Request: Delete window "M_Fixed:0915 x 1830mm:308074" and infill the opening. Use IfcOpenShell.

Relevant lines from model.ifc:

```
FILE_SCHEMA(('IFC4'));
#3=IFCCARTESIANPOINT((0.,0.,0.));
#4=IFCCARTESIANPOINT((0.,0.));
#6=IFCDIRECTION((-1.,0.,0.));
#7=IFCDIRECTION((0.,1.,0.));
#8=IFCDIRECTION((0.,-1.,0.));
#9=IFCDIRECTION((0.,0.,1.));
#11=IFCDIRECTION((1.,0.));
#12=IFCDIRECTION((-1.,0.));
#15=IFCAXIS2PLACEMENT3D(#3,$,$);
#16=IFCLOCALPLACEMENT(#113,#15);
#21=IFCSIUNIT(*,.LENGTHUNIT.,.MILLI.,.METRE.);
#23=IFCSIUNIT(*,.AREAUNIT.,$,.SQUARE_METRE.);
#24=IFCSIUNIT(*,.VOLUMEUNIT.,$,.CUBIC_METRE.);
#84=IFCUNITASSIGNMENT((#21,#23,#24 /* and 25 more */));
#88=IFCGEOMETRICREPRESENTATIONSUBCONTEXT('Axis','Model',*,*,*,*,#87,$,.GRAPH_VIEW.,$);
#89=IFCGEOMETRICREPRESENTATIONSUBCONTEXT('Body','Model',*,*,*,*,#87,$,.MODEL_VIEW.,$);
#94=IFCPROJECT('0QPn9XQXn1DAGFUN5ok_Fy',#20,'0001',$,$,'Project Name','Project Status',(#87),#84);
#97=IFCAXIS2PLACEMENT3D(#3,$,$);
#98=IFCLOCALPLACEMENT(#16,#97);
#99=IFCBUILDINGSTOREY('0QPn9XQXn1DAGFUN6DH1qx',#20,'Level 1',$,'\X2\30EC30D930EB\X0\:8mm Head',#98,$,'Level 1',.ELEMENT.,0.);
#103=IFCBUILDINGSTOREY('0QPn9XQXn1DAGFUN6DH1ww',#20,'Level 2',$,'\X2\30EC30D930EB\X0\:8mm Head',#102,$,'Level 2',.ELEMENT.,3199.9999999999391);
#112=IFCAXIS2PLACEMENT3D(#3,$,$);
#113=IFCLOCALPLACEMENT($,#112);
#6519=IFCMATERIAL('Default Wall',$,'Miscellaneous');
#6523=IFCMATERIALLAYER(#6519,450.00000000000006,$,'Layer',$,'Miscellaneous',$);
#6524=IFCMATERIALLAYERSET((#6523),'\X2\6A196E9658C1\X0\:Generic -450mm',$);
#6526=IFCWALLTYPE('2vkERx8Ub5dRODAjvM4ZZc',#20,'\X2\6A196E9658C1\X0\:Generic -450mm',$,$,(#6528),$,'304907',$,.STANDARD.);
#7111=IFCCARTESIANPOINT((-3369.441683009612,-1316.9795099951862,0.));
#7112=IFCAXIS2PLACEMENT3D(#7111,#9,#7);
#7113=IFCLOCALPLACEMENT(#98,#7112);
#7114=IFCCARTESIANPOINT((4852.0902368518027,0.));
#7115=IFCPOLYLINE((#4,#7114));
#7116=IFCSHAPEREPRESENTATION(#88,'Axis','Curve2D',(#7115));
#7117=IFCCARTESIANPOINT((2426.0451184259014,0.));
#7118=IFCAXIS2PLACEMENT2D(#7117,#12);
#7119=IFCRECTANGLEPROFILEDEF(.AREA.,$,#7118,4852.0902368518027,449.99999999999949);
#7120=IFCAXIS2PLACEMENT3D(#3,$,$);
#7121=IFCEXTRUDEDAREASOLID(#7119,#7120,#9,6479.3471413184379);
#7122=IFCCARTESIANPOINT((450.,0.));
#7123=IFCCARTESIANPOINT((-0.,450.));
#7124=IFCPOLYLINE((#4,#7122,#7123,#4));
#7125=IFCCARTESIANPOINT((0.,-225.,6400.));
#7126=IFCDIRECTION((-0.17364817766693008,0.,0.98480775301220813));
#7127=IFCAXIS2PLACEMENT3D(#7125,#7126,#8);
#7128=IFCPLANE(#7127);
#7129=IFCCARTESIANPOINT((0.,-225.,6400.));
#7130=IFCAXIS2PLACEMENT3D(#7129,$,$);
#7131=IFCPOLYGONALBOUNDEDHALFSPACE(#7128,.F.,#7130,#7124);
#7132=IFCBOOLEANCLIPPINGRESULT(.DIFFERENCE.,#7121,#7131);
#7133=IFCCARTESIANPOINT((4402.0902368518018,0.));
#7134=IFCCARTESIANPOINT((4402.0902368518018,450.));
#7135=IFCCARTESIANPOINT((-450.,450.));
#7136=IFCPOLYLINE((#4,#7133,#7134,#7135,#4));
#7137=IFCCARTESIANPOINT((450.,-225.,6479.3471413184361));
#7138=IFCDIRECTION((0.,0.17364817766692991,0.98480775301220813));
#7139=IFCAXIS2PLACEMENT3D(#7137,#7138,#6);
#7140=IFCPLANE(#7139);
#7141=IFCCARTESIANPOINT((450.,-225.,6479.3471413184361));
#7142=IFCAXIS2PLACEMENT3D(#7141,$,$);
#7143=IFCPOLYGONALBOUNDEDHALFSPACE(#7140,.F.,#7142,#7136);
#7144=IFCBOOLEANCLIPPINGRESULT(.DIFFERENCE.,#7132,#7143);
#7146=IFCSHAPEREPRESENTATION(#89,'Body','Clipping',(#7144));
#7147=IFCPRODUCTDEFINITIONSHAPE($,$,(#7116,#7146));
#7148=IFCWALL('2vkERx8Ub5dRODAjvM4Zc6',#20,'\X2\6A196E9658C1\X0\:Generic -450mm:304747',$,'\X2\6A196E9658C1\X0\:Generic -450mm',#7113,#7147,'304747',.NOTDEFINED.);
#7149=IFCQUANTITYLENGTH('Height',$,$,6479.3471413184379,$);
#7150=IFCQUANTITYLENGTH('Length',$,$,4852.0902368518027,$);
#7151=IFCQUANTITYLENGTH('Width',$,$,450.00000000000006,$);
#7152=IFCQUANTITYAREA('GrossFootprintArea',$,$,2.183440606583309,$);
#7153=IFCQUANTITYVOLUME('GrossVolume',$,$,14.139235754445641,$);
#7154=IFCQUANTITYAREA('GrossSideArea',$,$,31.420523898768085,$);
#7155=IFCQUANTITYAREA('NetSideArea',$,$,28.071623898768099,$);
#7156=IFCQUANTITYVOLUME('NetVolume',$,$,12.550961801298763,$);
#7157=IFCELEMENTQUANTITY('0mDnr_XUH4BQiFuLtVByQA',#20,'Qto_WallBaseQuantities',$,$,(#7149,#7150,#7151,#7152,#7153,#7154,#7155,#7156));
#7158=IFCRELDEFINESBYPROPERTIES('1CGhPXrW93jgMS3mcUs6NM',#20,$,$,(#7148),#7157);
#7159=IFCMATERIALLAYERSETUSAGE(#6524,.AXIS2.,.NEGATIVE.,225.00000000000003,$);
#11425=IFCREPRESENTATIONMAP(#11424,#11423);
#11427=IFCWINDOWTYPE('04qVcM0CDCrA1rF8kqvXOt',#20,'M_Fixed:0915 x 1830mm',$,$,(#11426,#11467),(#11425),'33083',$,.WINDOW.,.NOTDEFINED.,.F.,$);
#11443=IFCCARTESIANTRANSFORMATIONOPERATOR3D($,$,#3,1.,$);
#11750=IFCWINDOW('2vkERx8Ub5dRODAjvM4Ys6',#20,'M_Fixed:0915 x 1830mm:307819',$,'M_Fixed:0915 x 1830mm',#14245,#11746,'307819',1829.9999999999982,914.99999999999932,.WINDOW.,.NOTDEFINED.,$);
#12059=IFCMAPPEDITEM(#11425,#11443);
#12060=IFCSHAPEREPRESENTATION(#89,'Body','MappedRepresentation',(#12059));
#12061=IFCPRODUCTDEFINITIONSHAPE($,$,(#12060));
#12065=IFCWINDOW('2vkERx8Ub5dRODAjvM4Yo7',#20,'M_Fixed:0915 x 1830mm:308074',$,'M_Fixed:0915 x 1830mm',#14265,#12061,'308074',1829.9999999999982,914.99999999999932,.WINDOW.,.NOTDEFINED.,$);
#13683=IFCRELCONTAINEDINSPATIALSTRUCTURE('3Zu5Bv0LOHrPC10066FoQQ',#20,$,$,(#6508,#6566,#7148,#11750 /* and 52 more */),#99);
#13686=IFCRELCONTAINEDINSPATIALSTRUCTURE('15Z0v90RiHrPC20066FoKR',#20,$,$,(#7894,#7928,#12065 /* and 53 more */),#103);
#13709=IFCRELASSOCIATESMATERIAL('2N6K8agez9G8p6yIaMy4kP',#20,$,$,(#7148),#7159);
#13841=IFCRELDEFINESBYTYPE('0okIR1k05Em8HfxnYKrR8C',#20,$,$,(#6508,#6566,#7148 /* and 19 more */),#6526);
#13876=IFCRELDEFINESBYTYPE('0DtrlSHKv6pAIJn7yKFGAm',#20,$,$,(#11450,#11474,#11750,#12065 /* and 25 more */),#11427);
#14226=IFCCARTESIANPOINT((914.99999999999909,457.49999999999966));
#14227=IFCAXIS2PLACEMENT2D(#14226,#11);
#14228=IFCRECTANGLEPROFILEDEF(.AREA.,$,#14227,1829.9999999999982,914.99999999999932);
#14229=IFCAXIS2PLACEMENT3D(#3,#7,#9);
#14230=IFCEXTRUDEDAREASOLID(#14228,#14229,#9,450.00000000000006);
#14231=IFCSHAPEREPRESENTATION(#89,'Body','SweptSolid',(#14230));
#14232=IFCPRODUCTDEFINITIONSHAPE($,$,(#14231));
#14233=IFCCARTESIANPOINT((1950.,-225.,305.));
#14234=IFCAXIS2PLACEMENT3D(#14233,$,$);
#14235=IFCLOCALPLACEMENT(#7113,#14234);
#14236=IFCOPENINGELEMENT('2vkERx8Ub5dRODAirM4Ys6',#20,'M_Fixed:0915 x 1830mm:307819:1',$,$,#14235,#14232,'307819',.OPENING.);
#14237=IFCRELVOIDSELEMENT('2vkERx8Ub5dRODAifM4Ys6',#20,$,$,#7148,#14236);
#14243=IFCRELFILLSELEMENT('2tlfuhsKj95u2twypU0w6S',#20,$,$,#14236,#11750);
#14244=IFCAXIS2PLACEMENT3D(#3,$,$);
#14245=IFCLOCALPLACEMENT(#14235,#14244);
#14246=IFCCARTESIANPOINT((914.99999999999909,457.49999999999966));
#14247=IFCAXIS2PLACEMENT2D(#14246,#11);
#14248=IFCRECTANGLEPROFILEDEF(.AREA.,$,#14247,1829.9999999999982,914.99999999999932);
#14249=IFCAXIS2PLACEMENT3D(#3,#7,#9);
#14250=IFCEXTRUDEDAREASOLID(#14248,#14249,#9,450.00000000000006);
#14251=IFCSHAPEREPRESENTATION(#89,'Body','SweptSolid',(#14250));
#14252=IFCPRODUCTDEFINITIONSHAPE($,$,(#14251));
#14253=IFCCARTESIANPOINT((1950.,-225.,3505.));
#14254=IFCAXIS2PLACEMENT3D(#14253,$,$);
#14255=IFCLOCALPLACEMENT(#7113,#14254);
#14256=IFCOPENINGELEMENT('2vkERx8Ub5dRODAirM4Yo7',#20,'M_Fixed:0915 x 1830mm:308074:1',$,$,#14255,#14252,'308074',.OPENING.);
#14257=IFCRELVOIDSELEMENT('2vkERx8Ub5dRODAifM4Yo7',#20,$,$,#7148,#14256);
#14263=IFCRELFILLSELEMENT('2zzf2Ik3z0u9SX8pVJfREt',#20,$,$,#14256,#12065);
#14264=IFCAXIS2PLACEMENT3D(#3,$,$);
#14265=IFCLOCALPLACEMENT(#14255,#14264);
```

```python
import ifcopenshell
import ifcopenshell.api.feature
import ifcopenshell.api.pset
import ifcopenshell.api.root
import ifcopenshell.geom
import ifcopenshell.util.element
import ifcopenshell.util.shape
import ifcopenshell.util.unit

model = ifcopenshell.open("model.ifc")
area_scale = ifcopenshell.util.unit.calculate_unit_scale(model, "AREAUNIT")
volume_scale = ifcopenshell.util.unit.calculate_unit_scale(model, "VOLUMEUNIT")
settings = ifcopenshell.geom.settings()


def volume(element):
    """Net volume in cubic metres, openings subtracted."""
    shape = ifcopenshell.geom.create_shape(settings, element)
    return ifcopenshell.util.shape.get_volume(shape.geometry)


window = model.by_guid("2vkERx8Ub5dRODAjvM4Yo7")
opening = window.FillsVoids[0].RelatingOpeningElement
wall = opening.VoidsElements[0].RelatingBuildingElement
before = volume(wall)

ifcopenshell.api.root.remove_product(model, product=window)
ifcopenshell.api.feature.remove_feature(model, feature=opening)

after = volume(wall)
thickness = 0.45  # wall thickness in metres

# Update the wall's stored quantities.
qto = model.by_id(ifcopenshell.util.element.get_pset(wall, "Qto_WallBaseQuantities", should_inherit=False)["id"])
ifcopenshell.api.pset.edit_qto(model, qto=qto, properties={
    "NetSideArea": after / thickness / area_scale,
    "NetVolume": after / volume_scale,
})

print(f"wall volume {before:.3f} -> {after:.3f} m3")

model.write("model-out.ifc")
```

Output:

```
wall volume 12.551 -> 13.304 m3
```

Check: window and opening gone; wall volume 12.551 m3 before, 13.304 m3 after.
